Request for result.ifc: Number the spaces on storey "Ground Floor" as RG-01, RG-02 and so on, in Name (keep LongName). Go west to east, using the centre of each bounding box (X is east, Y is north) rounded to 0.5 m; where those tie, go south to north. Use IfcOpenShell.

First a look at what the model holds.

```python
import ifcopenshell
import ifcopenshell.util.element
import ifcopenshell.util.placement

model = ifcopenshell.open("result.ifc")
print(model.schema)
storey = next(s for s in model.by_type("IfcBuildingStorey") if s.Name == "Ground Floor")
spaces = [e for e in ifcopenshell.util.element.get_decomposition(storey) if e.is_a("IfcSpace")]
for e in sorted(spaces, key=lambda e: e.id()):
    origin = ifcopenshell.util.placement.get_local_placement(e.ObjectPlacement)[:3, 3]
    print(e.id(), e.Name, e.LongName, origin.round(2) + 0.0, sep=" | ")
```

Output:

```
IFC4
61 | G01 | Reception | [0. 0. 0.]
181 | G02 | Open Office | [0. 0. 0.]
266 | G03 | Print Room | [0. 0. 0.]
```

```python
import ifcopenshell
import ifcopenshell.geom
import ifcopenshell.util.element
import ifcopenshell.util.shape

model = ifcopenshell.open("result.ifc")
settings = ifcopenshell.geom.settings()
settings.set("use-world-coords", True)


def centre(element):
    shape = ifcopenshell.geom.create_shape(settings, element)
    return ifcopenshell.util.shape.get_bbox_centroid(shape.geometry)


storey = next(s for s in model.by_type("IfcBuildingStorey") if s.Name == "Ground Floor")
spaces = [e for e in ifcopenshell.util.element.get_decomposition(storey) if e.is_a("IfcSpace")]

# Insertion points can sit at a corner or the storey origin, so sort by the geometry (in metres).
centres = {e: centre(e) for e in spaces}
spaces.sort(key=lambda e: (round(centres[e][0] / 0.5), centres[e][1]))

for i, e in enumerate(spaces, start=1):
    number = f"RG-{i:02d}"
    e.Name = number
    print(e.id(), number)

model.write("result_edited.ifc")
```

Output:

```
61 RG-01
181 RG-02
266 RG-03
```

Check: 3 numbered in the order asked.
